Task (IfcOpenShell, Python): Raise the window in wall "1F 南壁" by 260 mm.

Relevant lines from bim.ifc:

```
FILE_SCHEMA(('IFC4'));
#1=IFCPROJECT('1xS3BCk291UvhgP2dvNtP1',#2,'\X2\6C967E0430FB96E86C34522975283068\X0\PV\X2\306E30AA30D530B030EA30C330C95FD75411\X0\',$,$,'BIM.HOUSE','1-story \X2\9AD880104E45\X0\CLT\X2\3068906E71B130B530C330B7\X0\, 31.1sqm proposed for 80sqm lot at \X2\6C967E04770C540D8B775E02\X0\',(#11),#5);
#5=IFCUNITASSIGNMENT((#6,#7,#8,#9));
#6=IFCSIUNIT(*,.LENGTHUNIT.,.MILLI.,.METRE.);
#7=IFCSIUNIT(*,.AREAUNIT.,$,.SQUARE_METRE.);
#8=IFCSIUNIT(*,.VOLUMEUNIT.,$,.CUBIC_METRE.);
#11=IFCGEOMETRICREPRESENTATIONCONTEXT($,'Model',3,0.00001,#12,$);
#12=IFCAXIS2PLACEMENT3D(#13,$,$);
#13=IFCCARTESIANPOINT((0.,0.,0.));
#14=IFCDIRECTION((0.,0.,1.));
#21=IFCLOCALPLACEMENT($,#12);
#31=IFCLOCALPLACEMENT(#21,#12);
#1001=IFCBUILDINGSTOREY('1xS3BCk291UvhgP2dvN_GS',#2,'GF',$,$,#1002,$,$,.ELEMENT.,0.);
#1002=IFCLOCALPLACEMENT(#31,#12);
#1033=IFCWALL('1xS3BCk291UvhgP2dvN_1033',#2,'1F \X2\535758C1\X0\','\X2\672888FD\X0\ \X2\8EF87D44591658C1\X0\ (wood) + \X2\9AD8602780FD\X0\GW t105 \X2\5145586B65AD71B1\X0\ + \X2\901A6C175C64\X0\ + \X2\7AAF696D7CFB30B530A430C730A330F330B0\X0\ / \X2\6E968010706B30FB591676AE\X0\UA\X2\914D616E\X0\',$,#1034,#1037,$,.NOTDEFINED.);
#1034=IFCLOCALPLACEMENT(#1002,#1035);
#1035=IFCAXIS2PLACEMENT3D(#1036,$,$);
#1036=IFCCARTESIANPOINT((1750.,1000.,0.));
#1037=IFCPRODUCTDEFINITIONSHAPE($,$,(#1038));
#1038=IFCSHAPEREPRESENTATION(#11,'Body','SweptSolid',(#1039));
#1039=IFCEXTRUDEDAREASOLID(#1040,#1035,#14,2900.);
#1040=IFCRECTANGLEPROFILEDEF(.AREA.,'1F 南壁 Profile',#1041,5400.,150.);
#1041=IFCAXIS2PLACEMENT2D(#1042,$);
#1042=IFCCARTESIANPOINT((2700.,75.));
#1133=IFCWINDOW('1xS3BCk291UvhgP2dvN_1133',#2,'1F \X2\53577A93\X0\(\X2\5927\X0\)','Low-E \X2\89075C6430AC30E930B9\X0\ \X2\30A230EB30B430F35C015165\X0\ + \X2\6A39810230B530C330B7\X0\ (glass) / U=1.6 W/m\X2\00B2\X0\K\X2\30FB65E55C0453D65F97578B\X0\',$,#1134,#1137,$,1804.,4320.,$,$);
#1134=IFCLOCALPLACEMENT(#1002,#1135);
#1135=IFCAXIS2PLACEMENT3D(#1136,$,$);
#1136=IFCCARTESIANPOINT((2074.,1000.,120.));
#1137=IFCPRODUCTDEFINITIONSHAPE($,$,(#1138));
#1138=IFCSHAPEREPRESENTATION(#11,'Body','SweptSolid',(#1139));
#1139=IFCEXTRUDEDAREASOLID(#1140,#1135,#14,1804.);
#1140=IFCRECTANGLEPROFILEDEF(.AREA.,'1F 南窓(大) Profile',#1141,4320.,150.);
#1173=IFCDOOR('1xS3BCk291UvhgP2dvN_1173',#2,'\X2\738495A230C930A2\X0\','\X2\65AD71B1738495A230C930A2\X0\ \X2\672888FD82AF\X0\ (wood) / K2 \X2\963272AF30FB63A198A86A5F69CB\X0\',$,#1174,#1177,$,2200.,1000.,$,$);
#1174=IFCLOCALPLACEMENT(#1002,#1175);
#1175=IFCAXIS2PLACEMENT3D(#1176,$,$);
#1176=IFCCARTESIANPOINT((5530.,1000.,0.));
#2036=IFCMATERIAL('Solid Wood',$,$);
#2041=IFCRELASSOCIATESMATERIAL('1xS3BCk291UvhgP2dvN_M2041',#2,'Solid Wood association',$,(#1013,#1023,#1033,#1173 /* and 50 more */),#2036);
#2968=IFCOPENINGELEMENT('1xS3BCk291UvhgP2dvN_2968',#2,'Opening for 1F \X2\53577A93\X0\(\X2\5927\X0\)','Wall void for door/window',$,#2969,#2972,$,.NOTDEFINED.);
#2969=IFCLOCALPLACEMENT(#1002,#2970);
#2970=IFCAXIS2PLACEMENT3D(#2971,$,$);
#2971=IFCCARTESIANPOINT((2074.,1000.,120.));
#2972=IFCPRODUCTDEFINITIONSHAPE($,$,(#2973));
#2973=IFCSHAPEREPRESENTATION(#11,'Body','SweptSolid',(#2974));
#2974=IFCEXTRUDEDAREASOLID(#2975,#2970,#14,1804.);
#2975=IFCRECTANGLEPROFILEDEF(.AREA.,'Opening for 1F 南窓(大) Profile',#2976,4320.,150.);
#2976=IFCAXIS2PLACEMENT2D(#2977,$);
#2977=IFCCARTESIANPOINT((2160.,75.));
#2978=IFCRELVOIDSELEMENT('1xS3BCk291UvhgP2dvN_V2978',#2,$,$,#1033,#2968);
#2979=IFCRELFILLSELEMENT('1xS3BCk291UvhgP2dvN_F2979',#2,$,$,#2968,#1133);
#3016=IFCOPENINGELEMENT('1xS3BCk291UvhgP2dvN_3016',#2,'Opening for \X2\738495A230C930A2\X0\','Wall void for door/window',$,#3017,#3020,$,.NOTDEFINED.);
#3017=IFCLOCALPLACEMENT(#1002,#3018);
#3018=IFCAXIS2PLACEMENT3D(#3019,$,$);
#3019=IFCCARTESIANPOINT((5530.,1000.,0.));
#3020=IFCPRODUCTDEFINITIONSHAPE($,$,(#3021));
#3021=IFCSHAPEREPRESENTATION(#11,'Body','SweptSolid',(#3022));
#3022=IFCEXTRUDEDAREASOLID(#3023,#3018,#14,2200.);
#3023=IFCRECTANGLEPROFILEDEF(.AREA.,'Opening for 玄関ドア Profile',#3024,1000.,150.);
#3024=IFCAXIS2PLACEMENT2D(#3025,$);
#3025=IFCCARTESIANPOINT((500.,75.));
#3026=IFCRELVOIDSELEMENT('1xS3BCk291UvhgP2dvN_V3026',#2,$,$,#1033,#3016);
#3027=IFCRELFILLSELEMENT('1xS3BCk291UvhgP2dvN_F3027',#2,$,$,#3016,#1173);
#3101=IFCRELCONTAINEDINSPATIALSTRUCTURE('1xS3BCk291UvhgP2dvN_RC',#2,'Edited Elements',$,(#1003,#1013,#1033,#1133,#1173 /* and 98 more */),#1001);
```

```python
import numpy as np
import ifcopenshell
import ifcopenshell.api.geometry
import ifcopenshell.util.placement
import ifcopenshell.util.unit

model = ifcopenshell.open("bim.ifc")
unit_scale = ifcopenshell.util.unit.calculate_unit_scale(model)

window = model.by_id(1133)
opening = window.FillsVoids[0].RelatingOpeningElement
dz = 0.26 / unit_scale

shift = np.array([0.0, 0.0, dz])
# The window is not placed relative to its opening, so move both.
for product in (opening, window):
    matrix = ifcopenshell.util.placement.get_local_placement(product.ObjectPlacement)
    matrix[:3, 3] += shift
    ifcopenshell.api.geometry.edit_object_placement(model, product=product, matrix=matrix, is_si=False)

print(f"moved by {dz * unit_scale:+.3f} m")

model.write("bim_rev.ifc")
```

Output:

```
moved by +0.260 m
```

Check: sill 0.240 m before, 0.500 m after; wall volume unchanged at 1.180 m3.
